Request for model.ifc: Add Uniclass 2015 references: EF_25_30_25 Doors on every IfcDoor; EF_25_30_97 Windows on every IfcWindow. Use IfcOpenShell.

First a look at what the model holds.

```python
import ifcopenshell

model = ifcopenshell.open("model.ifc")
print(model.schema)
print("classifications:", [c.Name for c in model.by_type("IfcClassification")])
for ifc_class in ("IfcDoor", "IfcRoof", "IfcStair", "IfcWall", "IfcWindow"):
    print(ifc_class, len(model.by_type(ifc_class)))
```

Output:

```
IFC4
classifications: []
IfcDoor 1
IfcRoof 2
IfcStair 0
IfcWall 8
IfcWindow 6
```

```python
import ifcopenshell
import ifcopenshell.api.classification

model = ifcopenshell.open("model.ifc")

system = ifcopenshell.api.classification.add_classification(model, classification="Uniclass 2015")

codes = {
    "IfcDoor": ("EF_25_30_25", "Doors"),
    "IfcWindow": ("EF_25_30_97", "Windows"),
}
for ifc_class, (code, name) in codes.items():
    products = model.by_type(ifc_class)
    ifcopenshell.api.classification.add_reference(
        model, products=products, classification=system, identification=code, name=name
    )
    print(code, len(products))

model.write("model_updated.ifc")
```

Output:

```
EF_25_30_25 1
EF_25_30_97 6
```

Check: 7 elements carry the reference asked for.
